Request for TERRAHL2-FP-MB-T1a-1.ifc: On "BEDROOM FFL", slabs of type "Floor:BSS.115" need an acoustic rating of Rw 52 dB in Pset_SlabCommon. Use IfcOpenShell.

First a look at what the model holds.

```python
import ifcopenshell
import ifcopenshell.util.element

model = ifcopenshell.open("TERRAHL2-FP-MB-T1a-1.ifc")
print(model.schema)
storey = next(s for s in model.by_type("IfcBuildingStorey") if s.Name == "BEDROOM FFL")
slabs = [e for e in ifcopenshell.util.element.get_decomposition(storey) if e.is_a("IfcSlab")]
seen = {}
for e in slabs:
    element_type = ifcopenshell.util.element.get_type(e)
    key = (element_type.Name if element_type != e and element_type else None, ifcopenshell.util.element.get_pset(e, "Pset_SlabCommon", "AcousticRating"))
    seen[key] = seen.get(key, 0) + 1
for (name, value), count in sorted(seen.items(), key=str):
    print(count, "x", name, "|", value)
```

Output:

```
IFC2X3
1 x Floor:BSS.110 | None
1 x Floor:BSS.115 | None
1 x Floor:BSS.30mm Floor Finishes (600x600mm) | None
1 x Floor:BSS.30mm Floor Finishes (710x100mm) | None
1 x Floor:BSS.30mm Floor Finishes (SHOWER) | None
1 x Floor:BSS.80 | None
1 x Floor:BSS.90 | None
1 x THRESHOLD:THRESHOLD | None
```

```python
import ifcopenshell
import ifcopenshell.api.pset
import ifcopenshell.util.element

model = ifcopenshell.open("TERRAHL2-FP-MB-T1a-1.ifc")

storey = next(s for s in model.by_type("IfcBuildingStorey") if s.Name == "BEDROOM FFL")
slabs = [e for e in ifcopenshell.util.element.get_decomposition(storey) if e.is_a("IfcSlab")]

count = 0
for e in slabs:
    element_type = ifcopenshell.util.element.get_type(e)
    if element_type in (None, e) or element_type.Name != "Floor:BSS.115":
        continue
    # add_pset returns the element's existing set when there is one.
    pset = ifcopenshell.api.pset.add_pset(model, product=e, name="Pset_SlabCommon")
    ifcopenshell.api.pset.edit_pset(model, pset=pset, properties={"AcousticRating": "Rw 52 dB"})
    count += 1

print(count, "slabs updated")

model.write("TERRAHL2-FP-MB-T1a-1_v2.ifc")
```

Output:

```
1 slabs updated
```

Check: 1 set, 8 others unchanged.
